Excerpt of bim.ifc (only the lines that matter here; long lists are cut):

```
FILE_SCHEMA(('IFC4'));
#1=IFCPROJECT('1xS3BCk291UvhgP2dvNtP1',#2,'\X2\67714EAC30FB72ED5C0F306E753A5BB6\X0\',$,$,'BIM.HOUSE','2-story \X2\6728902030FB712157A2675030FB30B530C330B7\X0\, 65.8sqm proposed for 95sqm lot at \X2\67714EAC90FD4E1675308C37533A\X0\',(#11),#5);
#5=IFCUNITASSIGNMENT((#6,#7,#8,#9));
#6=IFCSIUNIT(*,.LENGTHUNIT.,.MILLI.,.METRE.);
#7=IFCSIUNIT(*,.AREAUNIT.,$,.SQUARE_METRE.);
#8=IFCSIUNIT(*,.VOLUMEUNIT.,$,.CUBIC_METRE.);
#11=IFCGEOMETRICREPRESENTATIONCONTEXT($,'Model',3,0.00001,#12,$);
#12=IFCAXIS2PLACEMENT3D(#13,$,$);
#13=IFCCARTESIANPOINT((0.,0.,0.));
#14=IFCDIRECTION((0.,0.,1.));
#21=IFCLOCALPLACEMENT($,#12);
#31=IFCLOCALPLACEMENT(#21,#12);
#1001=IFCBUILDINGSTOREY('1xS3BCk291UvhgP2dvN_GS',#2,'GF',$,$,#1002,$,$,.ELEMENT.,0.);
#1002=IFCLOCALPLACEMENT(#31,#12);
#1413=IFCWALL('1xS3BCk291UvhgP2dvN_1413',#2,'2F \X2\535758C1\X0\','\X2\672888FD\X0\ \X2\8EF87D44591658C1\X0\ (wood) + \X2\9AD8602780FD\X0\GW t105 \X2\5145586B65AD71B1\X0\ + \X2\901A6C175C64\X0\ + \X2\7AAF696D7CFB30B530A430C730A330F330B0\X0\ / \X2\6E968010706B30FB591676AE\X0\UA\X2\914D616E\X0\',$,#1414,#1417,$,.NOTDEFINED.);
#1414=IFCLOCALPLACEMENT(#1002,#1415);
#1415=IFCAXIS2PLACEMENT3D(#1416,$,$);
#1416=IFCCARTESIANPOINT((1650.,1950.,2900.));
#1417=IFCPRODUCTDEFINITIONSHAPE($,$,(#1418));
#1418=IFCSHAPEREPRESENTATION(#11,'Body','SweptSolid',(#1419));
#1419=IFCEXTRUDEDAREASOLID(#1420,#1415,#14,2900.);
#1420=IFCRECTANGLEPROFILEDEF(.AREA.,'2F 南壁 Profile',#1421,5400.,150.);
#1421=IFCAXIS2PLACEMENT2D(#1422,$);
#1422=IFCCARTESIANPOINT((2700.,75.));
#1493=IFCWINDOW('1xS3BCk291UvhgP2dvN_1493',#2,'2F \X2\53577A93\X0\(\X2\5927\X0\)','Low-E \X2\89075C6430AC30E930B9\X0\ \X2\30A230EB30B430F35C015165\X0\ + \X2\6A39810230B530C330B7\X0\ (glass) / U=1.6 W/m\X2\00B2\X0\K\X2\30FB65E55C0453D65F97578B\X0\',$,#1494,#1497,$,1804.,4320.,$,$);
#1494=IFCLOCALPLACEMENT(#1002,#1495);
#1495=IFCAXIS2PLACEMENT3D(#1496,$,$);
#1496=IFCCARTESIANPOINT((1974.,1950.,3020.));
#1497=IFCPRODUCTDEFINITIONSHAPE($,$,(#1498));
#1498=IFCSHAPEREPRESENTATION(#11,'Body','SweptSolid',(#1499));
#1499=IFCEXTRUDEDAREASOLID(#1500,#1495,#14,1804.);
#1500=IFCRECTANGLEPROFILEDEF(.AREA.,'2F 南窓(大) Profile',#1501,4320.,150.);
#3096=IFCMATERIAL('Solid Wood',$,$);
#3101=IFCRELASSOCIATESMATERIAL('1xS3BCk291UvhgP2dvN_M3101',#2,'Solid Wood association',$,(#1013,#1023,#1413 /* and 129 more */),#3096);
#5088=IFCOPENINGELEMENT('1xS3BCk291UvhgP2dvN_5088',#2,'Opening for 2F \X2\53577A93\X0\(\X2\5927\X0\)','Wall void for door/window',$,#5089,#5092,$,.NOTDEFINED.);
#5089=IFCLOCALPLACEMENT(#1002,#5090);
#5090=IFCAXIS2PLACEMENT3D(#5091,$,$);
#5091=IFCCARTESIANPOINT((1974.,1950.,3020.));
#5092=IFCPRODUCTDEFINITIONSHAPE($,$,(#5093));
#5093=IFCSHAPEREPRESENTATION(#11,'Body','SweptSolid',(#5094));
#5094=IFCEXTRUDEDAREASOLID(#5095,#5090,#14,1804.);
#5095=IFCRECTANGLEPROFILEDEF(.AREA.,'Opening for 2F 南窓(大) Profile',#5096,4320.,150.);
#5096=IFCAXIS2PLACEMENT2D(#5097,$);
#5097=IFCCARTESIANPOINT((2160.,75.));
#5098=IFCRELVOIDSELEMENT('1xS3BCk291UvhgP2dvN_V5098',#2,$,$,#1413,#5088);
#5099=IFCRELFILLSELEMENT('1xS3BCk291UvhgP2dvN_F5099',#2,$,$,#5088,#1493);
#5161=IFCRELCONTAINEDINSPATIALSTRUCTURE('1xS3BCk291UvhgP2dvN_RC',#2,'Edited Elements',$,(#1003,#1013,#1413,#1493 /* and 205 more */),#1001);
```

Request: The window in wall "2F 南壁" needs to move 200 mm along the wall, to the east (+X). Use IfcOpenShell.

```python
import ifcopenshell
import ifcopenshell.api.geometry
import ifcopenshell.util.placement
import ifcopenshell.util.unit

model = ifcopenshell.open("bim.ifc")
unit_scale = ifcopenshell.util.unit.calculate_unit_scale(model)

window = model.by_id(1493)
opening = window.FillsVoids[0].RelatingOpeningElement
wall = opening.VoidsElements[0].RelatingBuildingElement

wall_matrix = ifcopenshell.util.placement.get_local_placement(wall.ObjectPlacement)
shift = wall_matrix[:3, 0] * 0.2 / unit_scale
before = ifcopenshell.util.placement.get_local_placement(window.ObjectPlacement)[:3, 3].copy()

# The window is not placed relative to its opening, so move both.
for product in (opening, window):
    matrix = ifcopenshell.util.placement.get_local_placement(product.ObjectPlacement)
    matrix[:3, 3] += shift
    ifcopenshell.api.geometry.edit_object_placement(model, product=product, matrix=matrix, is_si=False)

after = ifcopenshell.util.placement.get_local_placement(window.ObjectPlacement)[:3, 3]
print("window moved by", (after - before).round(3) + 0.0)

model.write("bim-out.ifc")
```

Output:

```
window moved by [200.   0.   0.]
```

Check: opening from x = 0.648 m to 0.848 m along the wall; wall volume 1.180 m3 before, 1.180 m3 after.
